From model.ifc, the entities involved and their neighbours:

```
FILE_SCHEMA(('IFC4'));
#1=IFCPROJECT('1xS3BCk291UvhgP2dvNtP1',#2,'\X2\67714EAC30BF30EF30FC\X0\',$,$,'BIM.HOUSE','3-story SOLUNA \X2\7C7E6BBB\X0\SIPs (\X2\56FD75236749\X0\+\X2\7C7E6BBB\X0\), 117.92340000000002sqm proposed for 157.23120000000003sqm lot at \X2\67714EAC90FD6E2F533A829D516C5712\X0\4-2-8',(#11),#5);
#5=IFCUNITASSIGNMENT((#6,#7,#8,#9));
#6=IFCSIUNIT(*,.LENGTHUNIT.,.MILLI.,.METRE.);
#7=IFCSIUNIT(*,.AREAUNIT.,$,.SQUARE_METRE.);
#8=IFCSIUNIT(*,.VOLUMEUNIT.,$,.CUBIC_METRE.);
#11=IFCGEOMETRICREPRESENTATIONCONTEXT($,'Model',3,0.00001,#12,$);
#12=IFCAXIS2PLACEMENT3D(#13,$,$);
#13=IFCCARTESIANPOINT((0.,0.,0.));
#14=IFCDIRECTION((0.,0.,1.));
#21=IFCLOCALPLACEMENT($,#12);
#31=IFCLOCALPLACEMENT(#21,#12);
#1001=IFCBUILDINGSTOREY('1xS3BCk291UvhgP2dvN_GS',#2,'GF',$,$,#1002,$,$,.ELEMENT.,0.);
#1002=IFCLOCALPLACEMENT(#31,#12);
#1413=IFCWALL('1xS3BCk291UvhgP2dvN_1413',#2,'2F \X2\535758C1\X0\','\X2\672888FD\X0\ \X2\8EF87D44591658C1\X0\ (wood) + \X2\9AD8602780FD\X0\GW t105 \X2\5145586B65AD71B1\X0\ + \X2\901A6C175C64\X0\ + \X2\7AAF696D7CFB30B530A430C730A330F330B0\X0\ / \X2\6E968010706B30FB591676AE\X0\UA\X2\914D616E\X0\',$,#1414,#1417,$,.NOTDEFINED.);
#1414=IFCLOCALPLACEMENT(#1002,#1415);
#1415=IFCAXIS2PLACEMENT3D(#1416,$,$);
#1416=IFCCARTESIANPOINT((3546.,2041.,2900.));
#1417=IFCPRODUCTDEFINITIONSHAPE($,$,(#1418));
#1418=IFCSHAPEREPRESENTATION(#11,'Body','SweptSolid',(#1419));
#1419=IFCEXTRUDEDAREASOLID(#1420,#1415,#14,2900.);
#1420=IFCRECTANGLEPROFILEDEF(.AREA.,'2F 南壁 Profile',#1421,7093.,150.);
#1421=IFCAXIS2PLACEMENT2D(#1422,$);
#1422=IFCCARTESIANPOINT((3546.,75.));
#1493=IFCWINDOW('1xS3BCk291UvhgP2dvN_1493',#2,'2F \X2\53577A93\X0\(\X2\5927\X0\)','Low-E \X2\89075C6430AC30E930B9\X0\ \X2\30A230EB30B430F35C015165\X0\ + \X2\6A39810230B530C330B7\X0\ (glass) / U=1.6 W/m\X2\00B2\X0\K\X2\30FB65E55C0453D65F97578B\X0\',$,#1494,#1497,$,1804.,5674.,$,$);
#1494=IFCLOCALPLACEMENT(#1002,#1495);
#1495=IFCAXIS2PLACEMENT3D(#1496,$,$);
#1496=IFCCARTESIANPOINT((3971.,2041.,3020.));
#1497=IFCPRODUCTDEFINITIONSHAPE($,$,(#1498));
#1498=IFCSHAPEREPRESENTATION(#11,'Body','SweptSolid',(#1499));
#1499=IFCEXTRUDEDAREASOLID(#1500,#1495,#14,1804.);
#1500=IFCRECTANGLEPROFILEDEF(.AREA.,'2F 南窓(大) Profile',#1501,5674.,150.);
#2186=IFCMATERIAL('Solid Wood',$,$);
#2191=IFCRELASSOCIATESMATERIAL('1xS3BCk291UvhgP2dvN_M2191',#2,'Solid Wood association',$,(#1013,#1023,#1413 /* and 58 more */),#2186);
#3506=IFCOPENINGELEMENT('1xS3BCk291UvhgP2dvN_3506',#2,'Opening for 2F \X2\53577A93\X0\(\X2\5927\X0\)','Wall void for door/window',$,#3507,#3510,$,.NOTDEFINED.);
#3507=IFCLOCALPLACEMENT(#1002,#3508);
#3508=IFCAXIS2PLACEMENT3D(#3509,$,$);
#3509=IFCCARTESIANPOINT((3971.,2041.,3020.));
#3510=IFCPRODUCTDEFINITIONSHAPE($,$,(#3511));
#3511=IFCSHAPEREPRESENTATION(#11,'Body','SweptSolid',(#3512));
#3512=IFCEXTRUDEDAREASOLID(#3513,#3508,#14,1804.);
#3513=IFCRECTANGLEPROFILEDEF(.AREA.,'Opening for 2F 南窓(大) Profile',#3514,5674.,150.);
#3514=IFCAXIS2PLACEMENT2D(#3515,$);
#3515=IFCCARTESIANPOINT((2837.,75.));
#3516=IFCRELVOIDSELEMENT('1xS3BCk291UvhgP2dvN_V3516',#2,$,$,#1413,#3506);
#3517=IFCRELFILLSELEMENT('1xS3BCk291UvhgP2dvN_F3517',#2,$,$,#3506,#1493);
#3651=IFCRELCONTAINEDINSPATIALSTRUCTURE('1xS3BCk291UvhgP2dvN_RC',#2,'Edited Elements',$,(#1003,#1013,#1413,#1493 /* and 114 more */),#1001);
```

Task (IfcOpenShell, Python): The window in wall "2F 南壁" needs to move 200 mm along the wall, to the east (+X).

```python
import ifcopenshell
import ifcopenshell.api.geometry
import ifcopenshell.util.placement

model = ifcopenshell.open("model.ifc")

window = model.by_guid("1xS3BCk291UvhgP2dvN_1493")
opening = window.FillsVoids[0].RelatingOpeningElement
wall = opening.VoidsElements[0].RelatingBuildingElement

wall_matrix = ifcopenshell.util.placement.get_local_placement(wall.ObjectPlacement)
shift = wall_matrix[:3, 0] * 200.0
before = ifcopenshell.util.placement.get_local_placement(window.ObjectPlacement)[:3, 3].copy()

# The window is not placed relative to its opening, so move both.
for product in (opening, window):
    matrix = ifcopenshell.util.placement.get_local_placement(product.ObjectPlacement)
    matrix[:3, 3] += shift
    ifcopenshell.api.geometry.edit_object_placement(model, product=product, matrix=matrix, is_si=False)

after = ifcopenshell.util.placement.get_local_placement(window.ObjectPlacement)[:3, 3]
print("window moved by", (after - before).round(3) + 0.0)

model.write("model_updated.ifc")
```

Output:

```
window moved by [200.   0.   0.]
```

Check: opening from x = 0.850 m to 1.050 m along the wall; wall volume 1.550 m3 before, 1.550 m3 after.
